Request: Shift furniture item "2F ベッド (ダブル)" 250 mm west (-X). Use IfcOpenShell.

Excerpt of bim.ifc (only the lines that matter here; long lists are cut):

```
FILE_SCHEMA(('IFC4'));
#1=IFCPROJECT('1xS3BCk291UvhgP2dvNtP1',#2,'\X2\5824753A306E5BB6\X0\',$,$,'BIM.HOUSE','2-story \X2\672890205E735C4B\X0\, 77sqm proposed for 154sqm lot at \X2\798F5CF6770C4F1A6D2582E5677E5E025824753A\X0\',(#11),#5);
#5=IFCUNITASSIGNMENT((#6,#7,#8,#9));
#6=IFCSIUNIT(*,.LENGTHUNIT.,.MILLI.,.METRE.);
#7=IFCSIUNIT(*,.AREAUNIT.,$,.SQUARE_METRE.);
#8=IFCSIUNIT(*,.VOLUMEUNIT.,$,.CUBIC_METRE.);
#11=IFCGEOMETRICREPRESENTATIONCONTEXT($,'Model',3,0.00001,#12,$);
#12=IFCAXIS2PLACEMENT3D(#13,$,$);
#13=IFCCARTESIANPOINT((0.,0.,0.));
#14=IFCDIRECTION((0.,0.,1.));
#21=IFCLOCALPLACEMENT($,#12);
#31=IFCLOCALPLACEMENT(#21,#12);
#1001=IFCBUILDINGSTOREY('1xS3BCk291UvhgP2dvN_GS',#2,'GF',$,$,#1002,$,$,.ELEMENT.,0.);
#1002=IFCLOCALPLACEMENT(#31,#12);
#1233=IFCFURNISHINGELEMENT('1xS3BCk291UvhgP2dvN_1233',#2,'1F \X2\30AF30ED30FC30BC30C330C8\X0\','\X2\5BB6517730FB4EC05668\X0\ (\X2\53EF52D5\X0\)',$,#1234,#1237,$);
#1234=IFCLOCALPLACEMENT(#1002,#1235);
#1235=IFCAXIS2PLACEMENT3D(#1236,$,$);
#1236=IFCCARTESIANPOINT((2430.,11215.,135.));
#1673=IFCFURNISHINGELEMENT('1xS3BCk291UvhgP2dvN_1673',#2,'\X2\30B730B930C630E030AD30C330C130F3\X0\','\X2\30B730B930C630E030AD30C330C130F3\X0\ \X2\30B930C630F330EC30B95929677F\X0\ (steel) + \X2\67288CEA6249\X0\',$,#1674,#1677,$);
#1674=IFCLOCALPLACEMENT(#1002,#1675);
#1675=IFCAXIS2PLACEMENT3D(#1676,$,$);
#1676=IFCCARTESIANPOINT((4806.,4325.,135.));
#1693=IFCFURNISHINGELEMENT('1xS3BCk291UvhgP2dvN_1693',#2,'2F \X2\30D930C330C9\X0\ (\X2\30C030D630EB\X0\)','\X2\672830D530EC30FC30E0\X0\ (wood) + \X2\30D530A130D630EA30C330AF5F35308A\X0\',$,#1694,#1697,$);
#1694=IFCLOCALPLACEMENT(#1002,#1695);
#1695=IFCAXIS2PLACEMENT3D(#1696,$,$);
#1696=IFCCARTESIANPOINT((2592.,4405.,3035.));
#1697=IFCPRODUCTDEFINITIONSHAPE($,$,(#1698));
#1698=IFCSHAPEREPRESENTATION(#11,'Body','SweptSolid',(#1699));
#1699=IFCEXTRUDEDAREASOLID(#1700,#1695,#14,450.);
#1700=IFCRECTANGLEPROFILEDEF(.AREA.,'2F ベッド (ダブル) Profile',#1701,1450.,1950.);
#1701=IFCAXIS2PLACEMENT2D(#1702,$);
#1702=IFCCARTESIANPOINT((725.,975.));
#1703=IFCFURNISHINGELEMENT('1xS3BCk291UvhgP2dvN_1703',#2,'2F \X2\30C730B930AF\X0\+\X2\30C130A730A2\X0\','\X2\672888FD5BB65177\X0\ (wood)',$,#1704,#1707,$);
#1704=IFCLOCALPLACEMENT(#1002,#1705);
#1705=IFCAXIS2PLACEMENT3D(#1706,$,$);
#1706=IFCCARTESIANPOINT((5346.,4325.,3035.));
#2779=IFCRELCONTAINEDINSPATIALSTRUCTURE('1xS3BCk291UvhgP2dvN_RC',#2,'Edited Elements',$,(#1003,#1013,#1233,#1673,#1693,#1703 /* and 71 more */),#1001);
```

```python
import ifcopenshell
import ifcopenshell.api.geometry
import ifcopenshell.util.placement
import ifcopenshell.util.unit

model = ifcopenshell.open("bim.ifc")
unit_scale = ifcopenshell.util.unit.calculate_unit_scale(model)

item = model.by_id(1693)
matrix = ifcopenshell.util.placement.get_local_placement(item.ObjectPlacement)
matrix[0, 3] -= 0.25 / unit_scale
ifcopenshell.api.geometry.edit_object_placement(model, product=item, matrix=matrix, is_si=False)

print(ifcopenshell.util.placement.get_local_placement(item.ObjectPlacement).round(3) + 0.0)

model.write("bim_rev.ifc")
```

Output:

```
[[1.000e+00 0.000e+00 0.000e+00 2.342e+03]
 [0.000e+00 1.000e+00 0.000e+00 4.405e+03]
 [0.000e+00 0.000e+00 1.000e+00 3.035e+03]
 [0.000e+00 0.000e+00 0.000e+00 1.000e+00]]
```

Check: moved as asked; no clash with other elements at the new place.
